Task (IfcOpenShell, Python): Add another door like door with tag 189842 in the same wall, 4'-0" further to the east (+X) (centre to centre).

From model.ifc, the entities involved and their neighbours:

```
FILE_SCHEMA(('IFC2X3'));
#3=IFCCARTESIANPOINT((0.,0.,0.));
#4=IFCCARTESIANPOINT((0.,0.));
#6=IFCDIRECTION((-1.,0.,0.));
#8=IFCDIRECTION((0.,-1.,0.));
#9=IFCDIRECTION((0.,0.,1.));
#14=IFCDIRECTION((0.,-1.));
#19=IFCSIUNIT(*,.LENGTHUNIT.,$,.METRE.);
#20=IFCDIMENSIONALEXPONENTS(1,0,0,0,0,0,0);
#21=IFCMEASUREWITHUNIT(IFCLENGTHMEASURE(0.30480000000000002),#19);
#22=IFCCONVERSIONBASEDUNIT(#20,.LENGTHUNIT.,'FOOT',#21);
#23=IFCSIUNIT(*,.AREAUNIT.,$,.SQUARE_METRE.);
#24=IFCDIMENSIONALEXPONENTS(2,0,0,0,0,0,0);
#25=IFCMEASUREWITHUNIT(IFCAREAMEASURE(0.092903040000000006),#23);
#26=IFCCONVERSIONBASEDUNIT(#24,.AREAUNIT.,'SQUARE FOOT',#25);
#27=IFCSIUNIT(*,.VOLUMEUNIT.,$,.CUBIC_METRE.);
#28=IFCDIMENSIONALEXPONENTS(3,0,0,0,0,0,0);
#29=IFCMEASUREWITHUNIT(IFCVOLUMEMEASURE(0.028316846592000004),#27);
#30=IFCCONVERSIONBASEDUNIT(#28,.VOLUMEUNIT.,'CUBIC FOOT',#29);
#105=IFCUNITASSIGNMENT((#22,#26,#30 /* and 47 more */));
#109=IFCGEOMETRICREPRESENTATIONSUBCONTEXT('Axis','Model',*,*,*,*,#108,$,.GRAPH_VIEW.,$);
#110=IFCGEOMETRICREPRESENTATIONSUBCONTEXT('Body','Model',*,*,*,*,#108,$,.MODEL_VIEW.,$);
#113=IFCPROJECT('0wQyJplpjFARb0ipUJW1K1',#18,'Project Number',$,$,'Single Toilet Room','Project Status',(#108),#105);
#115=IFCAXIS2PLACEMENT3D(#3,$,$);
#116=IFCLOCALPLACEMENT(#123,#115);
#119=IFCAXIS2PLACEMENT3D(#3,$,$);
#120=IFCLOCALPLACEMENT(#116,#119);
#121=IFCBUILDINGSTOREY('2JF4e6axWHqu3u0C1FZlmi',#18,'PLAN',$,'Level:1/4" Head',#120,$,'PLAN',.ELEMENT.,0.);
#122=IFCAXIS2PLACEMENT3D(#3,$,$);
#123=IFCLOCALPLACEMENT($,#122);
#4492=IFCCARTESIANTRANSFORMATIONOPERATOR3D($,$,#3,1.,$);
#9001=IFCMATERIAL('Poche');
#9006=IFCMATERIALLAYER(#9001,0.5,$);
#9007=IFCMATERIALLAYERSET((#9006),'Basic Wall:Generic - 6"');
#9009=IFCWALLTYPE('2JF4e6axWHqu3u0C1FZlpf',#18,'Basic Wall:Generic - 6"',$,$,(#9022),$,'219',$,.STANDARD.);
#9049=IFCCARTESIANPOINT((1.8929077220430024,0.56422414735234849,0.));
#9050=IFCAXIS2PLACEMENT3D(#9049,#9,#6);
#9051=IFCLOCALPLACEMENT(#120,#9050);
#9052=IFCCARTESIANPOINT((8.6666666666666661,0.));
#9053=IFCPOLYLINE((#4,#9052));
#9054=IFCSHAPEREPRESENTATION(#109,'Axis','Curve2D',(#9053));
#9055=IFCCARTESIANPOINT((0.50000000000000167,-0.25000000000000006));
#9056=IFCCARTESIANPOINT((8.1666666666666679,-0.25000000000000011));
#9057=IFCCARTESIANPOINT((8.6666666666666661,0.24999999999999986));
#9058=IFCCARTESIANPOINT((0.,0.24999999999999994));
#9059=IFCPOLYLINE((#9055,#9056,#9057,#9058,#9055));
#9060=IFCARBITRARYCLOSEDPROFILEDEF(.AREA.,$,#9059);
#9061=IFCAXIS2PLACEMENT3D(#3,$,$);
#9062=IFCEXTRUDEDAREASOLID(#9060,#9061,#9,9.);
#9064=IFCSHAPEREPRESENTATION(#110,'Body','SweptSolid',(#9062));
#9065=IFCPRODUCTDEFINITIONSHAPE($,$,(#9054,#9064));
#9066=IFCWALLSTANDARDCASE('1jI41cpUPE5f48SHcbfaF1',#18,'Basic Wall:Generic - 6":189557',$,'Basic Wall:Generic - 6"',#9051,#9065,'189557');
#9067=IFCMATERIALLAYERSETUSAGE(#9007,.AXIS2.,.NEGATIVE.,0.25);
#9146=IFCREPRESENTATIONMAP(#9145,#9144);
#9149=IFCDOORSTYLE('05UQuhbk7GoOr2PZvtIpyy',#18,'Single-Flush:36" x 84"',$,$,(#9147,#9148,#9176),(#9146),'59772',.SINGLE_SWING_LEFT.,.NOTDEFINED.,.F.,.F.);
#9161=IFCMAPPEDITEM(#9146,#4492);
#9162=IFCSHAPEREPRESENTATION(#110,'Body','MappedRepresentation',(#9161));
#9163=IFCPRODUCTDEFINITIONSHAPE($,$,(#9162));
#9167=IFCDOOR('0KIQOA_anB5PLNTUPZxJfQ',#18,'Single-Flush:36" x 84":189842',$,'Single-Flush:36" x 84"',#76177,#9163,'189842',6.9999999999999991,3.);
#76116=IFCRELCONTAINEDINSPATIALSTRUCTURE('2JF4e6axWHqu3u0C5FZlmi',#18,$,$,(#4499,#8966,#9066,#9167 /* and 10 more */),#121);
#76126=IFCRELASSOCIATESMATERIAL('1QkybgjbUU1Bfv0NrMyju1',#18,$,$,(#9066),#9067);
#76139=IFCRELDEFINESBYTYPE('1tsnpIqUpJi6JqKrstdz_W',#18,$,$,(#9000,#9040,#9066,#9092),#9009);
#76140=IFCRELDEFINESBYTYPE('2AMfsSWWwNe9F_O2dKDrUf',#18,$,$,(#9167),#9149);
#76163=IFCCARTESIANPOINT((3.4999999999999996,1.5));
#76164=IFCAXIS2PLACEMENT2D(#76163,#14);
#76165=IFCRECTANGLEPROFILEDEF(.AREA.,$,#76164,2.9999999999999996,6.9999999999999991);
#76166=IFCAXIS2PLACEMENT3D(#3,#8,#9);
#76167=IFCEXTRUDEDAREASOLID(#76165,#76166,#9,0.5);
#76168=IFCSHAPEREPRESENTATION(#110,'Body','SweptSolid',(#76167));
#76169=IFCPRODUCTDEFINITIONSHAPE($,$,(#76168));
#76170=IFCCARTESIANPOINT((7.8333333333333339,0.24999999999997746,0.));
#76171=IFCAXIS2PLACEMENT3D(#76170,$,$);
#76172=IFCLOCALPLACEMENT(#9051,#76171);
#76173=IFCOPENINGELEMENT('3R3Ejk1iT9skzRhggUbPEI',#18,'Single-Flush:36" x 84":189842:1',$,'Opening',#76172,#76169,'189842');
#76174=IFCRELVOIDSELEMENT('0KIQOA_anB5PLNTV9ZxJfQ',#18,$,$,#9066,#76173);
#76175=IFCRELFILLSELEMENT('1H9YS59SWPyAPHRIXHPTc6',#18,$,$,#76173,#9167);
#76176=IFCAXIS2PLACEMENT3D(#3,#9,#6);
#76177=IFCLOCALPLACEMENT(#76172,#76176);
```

```python
import ifcopenshell
import ifcopenshell.api.feature
import ifcopenshell.api.geometry
import ifcopenshell.api.root
import ifcopenshell.geom
import ifcopenshell.util.element
import ifcopenshell.util.placement
import ifcopenshell.util.shape
import ifcopenshell.util.unit

model = ifcopenshell.open("model.ifc")
unit_scale = ifcopenshell.util.unit.calculate_unit_scale(model)
settings = ifcopenshell.geom.settings()


def volume(element):
    """Net volume in cubic metres, openings subtracted."""
    shape = ifcopenshell.geom.create_shape(settings, element)
    return ifcopenshell.util.shape.get_volume(shape.geometry)


def reuse_history(source, copy):
    """copy_class also copies each property set's owner history, people and application; keep the originals."""
    for rel in copy.IsDefinedBy:
        if rel.is_a("IfcRelDefinesByProperties") and (history := rel.RelatingPropertyDefinition.OwnerHistory):
            rel.RelatingPropertyDefinition.OwnerHistory = source.OwnerHistory
            ifcopenshell.util.element.remove_deep2(model, history)


door = model.by_guid("0KIQOA_anB5PLNTUPZxJfQ")
opening = door.FillsVoids[0].RelatingOpeningElement
wall = opening.VoidsElements[0].RelatingBuildingElement
before = volume(wall)
shift = ifcopenshell.util.placement.get_local_placement(wall.ObjectPlacement)[:3, 0] * -48 * 0.0254 / unit_scale

# copy_class copies the void relationship, type, container and properties, but no geometry.
new_opening = ifcopenshell.api.root.copy_class(model, product=opening)
new_opening.Representation = ifcopenshell.util.element.copy_deep(
    model, opening.Representation, exclude=["IfcGeometricRepresentationContext", "IfcRepresentationMap"]
)
new_opening.Name = 'Single-Flush:36" x 84"'
new_opening.Tag = None
new_door = ifcopenshell.api.root.copy_class(model, product=door)
new_door.Representation = ifcopenshell.util.element.copy_deep(
    model, door.Representation, exclude=["IfcGeometricRepresentationContext", "IfcRepresentationMap"]
)
new_door.Name = 'Single-Flush:36" x 84"'
new_door.Tag = None
reuse_history(door, new_door)
fills = ifcopenshell.api.feature.add_filling(model, opening=new_opening, element=new_door)
fills.OwnerHistory = new_door.OwnerHistory  # required in IFC2X3

for old, new in ((opening, new_opening), (door, new_door)):
    matrix = ifcopenshell.util.placement.get_local_placement(old.ObjectPlacement)
    matrix[:3, 3] += shift
    ifcopenshell.api.geometry.edit_object_placement(model, product=new, matrix=matrix, is_si=False)

after = volume(wall)

print(f"wall volume {before:.3f} -> {after:.3f} m3")

model.write("model-out.ifc")
```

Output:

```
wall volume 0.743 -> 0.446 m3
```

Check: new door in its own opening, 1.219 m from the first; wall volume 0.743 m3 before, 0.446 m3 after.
